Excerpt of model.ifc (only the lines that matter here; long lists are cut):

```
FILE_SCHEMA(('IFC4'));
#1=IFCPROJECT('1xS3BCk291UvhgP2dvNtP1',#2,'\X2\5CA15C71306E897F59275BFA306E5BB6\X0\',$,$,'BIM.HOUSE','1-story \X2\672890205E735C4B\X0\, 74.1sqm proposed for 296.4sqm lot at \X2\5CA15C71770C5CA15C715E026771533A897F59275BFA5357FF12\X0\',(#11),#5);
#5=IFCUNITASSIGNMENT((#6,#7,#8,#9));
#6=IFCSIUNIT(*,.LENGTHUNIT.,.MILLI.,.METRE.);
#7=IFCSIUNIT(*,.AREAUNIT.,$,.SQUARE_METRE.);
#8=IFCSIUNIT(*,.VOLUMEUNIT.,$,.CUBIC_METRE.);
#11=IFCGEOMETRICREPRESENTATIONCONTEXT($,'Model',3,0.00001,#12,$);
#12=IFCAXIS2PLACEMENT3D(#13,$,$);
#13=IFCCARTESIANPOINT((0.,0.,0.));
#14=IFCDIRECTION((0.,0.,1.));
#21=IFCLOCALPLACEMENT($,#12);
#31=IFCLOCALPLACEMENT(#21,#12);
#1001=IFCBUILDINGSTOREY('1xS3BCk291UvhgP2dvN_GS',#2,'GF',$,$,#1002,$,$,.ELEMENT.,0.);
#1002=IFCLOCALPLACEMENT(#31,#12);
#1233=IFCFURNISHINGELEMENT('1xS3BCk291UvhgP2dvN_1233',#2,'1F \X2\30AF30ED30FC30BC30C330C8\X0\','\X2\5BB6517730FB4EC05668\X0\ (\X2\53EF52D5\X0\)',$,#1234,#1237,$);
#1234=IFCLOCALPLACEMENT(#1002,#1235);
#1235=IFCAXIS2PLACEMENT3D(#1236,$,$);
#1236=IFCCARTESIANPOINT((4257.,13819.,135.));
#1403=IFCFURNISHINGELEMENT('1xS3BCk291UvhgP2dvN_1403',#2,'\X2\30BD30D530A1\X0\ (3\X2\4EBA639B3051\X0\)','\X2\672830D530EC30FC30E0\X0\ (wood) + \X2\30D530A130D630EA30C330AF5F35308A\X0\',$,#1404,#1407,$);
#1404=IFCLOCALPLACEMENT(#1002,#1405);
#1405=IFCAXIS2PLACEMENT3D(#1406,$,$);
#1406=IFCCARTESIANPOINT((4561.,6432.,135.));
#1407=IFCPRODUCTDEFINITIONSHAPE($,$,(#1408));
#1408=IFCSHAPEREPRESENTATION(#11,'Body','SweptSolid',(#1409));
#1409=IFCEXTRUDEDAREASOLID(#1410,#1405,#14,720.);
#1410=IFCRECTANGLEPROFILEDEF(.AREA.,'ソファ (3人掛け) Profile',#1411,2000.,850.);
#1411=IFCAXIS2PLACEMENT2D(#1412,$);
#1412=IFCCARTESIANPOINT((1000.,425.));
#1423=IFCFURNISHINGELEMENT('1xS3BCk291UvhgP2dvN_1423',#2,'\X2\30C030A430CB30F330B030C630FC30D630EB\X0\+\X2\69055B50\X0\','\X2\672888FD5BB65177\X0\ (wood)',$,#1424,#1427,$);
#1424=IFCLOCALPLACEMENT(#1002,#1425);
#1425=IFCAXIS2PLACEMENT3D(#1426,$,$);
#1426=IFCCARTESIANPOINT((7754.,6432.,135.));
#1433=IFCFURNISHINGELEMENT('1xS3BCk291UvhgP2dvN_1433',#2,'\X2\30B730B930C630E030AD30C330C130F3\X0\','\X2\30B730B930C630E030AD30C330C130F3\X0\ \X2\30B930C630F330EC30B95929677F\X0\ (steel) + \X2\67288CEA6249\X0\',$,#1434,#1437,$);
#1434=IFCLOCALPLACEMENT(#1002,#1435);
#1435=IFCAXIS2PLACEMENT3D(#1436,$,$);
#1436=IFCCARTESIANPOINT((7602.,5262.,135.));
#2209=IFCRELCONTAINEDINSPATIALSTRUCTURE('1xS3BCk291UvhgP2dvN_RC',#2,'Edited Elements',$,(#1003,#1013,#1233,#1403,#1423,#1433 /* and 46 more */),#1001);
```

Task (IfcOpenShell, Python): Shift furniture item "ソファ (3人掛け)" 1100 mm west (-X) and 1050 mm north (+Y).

```python
import ifcopenshell
import ifcopenshell.api.geometry
import ifcopenshell.util.placement
import ifcopenshell.util.unit

model = ifcopenshell.open("model.ifc")
unit_scale = ifcopenshell.util.unit.calculate_unit_scale(model)

item = model.by_id(1403)
matrix = ifcopenshell.util.placement.get_local_placement(item.ObjectPlacement)
matrix[0, 3] -= 1.1 / unit_scale
matrix[1, 3] += 1.05 / unit_scale
ifcopenshell.api.geometry.edit_object_placement(model, product=item, matrix=matrix, is_si=False)

print(ifcopenshell.util.placement.get_local_placement(item.ObjectPlacement).round(3) + 0.0)

model.write("model_edited.ifc")
```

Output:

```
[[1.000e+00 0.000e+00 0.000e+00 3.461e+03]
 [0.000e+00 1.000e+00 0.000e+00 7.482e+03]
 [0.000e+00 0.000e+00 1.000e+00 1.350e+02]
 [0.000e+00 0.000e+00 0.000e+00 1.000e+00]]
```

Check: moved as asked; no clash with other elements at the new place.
